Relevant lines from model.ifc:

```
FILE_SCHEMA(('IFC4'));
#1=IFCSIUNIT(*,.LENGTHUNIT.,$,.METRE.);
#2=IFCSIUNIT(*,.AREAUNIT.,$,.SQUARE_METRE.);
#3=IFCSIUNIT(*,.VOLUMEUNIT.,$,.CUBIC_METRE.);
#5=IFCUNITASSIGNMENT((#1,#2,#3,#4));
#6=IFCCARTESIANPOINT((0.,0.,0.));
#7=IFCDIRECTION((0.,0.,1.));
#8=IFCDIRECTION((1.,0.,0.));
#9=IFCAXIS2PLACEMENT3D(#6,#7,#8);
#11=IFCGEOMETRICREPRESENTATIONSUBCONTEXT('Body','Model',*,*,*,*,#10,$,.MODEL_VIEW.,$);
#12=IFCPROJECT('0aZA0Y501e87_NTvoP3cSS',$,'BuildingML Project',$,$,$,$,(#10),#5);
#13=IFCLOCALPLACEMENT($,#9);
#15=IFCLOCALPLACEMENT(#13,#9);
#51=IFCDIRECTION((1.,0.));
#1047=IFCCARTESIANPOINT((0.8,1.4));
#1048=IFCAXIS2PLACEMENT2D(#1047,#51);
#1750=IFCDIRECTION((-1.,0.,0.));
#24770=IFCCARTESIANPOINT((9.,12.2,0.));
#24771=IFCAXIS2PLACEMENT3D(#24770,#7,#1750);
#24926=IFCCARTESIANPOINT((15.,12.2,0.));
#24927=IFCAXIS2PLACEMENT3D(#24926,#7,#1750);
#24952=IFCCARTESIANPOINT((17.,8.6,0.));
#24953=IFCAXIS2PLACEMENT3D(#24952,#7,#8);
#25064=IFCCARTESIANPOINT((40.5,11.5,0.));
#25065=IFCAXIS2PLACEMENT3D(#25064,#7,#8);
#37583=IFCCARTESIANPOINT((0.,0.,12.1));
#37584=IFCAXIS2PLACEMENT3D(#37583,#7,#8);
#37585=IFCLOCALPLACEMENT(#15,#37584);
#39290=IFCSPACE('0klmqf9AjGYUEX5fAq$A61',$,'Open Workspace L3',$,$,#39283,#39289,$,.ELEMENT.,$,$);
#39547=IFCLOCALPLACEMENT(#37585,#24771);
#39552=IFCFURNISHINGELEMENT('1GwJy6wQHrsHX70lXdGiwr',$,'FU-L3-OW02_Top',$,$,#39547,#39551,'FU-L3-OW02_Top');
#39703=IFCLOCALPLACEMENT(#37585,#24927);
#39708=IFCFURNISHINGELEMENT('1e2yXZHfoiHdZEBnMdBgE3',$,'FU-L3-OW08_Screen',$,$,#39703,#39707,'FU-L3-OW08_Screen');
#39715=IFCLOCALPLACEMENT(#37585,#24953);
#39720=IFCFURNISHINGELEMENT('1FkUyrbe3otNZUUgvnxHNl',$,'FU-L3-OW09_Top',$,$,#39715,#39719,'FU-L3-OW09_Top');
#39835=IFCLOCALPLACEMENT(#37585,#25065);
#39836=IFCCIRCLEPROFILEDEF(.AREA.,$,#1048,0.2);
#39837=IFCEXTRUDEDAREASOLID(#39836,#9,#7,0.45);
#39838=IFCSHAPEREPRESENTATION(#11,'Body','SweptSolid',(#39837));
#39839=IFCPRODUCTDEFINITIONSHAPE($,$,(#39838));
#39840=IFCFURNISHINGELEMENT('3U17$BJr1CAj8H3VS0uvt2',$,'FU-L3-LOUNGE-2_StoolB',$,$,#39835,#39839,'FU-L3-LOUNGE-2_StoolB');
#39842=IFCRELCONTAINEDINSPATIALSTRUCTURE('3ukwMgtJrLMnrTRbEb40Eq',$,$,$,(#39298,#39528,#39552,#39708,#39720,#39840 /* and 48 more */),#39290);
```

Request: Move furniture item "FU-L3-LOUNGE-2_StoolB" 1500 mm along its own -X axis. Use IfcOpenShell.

```python
import ifcopenshell
import ifcopenshell.api.geometry
import ifcopenshell.util.placement
import ifcopenshell.util.unit

model = ifcopenshell.open("model.ifc")
unit_scale = ifcopenshell.util.unit.calculate_unit_scale(model)

item = model.by_guid("3U17$BJr1CAj8H3VS0uvt2")
matrix = ifcopenshell.util.placement.get_local_placement(item.ObjectPlacement)
matrix[:3, 3] -= matrix[:3, 0] * 1.5 / unit_scale
ifcopenshell.api.geometry.edit_object_placement(model, product=item, matrix=matrix, is_si=False)

print(ifcopenshell.util.placement.get_local_placement(item.ObjectPlacement).round(3) + 0.0)

model.write("model-out.ifc")
```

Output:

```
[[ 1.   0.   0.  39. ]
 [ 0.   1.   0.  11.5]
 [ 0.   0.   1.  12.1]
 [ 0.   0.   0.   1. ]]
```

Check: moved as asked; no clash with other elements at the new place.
